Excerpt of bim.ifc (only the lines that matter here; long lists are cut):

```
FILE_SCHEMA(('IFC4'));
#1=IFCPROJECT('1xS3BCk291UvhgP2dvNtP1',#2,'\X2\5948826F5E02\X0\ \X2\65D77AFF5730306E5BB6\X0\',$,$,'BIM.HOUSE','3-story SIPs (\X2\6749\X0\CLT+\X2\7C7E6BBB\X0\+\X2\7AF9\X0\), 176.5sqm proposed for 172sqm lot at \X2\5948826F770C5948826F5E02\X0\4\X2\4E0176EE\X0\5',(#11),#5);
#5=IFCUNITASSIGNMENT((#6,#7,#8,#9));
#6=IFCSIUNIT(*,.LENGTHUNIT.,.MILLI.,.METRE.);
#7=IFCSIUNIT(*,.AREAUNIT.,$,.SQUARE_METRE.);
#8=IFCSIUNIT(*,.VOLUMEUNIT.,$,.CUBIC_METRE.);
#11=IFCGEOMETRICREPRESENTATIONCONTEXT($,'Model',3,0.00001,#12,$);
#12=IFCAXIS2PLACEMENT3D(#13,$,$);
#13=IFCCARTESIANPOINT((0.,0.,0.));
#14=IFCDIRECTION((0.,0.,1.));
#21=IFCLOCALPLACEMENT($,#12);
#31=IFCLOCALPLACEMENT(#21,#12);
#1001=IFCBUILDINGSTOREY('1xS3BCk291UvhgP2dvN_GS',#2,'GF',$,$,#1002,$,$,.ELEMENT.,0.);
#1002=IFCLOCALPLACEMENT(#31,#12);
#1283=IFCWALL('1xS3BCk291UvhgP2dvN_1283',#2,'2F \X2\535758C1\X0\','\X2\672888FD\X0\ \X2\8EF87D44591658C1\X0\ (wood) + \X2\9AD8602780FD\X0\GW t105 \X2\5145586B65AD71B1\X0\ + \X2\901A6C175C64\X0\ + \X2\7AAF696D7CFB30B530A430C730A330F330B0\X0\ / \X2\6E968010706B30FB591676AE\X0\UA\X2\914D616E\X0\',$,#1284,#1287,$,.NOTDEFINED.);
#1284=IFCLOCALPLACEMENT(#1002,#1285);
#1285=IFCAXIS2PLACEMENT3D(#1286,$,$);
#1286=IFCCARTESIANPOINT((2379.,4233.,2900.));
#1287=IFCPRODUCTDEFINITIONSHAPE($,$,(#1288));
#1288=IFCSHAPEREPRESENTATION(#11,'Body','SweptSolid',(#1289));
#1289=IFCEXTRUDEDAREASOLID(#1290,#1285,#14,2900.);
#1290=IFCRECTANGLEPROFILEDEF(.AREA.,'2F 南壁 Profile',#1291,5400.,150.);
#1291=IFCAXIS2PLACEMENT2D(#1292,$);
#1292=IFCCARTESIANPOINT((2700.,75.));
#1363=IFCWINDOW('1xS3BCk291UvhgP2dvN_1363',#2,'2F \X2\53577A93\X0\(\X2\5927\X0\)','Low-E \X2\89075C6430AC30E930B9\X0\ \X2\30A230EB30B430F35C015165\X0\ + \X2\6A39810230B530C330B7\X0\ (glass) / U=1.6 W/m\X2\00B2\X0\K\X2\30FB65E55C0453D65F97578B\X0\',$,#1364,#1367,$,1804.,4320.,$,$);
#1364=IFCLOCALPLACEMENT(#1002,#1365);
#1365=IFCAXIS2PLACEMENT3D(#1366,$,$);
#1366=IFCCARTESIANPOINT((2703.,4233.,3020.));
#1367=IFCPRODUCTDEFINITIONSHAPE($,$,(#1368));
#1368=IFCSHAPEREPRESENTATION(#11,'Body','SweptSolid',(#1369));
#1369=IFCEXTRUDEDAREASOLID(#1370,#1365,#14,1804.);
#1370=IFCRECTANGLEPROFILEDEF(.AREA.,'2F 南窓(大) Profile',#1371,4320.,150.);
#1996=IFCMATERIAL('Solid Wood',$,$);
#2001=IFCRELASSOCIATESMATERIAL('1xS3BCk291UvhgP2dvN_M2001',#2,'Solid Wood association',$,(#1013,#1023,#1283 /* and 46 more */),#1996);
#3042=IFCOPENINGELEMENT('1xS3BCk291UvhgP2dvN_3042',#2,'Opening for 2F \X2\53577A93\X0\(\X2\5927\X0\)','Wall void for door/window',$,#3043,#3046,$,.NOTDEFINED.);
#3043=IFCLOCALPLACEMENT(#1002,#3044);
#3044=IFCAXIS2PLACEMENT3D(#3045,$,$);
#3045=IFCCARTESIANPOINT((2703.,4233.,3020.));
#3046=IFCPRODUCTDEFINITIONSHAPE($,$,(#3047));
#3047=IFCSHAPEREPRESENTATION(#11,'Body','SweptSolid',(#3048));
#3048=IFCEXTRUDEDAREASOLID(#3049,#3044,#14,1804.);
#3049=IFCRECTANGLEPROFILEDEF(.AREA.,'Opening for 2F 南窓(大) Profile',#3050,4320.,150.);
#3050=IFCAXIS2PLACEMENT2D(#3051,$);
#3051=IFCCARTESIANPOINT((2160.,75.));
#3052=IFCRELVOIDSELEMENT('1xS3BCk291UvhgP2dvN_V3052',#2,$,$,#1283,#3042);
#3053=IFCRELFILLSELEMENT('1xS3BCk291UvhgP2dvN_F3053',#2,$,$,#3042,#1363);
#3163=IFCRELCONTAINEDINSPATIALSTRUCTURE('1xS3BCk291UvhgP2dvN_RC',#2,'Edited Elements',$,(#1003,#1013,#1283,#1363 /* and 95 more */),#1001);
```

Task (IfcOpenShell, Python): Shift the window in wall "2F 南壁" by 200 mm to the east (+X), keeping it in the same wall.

```python
import ifcopenshell
import ifcopenshell.api.geometry
import ifcopenshell.util.placement
import ifcopenshell.util.unit

model = ifcopenshell.open("bim.ifc")
unit_scale = ifcopenshell.util.unit.calculate_unit_scale(model)

window = model.by_id(1363)
opening = window.FillsVoids[0].RelatingOpeningElement
wall = opening.VoidsElements[0].RelatingBuildingElement

wall_matrix = ifcopenshell.util.placement.get_local_placement(wall.ObjectPlacement)
shift = wall_matrix[:3, 0] * 0.2 / unit_scale
before = ifcopenshell.util.placement.get_local_placement(window.ObjectPlacement)[:3, 3].copy()

# The window is not placed relative to its opening, so move both.
for product in (opening, window):
    matrix = ifcopenshell.util.placement.get_local_placement(product.ObjectPlacement)
    matrix[:3, 3] += shift
    ifcopenshell.api.geometry.edit_object_placement(model, product=product, matrix=matrix, is_si=False)

after = ifcopenshell.util.placement.get_local_placement(window.ObjectPlacement)[:3, 3]
print("window moved by", (after - before).round(3) + 0.0)

model.write("bim-out.ifc")
```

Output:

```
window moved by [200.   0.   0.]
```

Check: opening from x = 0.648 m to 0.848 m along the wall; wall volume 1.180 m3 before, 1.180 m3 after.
